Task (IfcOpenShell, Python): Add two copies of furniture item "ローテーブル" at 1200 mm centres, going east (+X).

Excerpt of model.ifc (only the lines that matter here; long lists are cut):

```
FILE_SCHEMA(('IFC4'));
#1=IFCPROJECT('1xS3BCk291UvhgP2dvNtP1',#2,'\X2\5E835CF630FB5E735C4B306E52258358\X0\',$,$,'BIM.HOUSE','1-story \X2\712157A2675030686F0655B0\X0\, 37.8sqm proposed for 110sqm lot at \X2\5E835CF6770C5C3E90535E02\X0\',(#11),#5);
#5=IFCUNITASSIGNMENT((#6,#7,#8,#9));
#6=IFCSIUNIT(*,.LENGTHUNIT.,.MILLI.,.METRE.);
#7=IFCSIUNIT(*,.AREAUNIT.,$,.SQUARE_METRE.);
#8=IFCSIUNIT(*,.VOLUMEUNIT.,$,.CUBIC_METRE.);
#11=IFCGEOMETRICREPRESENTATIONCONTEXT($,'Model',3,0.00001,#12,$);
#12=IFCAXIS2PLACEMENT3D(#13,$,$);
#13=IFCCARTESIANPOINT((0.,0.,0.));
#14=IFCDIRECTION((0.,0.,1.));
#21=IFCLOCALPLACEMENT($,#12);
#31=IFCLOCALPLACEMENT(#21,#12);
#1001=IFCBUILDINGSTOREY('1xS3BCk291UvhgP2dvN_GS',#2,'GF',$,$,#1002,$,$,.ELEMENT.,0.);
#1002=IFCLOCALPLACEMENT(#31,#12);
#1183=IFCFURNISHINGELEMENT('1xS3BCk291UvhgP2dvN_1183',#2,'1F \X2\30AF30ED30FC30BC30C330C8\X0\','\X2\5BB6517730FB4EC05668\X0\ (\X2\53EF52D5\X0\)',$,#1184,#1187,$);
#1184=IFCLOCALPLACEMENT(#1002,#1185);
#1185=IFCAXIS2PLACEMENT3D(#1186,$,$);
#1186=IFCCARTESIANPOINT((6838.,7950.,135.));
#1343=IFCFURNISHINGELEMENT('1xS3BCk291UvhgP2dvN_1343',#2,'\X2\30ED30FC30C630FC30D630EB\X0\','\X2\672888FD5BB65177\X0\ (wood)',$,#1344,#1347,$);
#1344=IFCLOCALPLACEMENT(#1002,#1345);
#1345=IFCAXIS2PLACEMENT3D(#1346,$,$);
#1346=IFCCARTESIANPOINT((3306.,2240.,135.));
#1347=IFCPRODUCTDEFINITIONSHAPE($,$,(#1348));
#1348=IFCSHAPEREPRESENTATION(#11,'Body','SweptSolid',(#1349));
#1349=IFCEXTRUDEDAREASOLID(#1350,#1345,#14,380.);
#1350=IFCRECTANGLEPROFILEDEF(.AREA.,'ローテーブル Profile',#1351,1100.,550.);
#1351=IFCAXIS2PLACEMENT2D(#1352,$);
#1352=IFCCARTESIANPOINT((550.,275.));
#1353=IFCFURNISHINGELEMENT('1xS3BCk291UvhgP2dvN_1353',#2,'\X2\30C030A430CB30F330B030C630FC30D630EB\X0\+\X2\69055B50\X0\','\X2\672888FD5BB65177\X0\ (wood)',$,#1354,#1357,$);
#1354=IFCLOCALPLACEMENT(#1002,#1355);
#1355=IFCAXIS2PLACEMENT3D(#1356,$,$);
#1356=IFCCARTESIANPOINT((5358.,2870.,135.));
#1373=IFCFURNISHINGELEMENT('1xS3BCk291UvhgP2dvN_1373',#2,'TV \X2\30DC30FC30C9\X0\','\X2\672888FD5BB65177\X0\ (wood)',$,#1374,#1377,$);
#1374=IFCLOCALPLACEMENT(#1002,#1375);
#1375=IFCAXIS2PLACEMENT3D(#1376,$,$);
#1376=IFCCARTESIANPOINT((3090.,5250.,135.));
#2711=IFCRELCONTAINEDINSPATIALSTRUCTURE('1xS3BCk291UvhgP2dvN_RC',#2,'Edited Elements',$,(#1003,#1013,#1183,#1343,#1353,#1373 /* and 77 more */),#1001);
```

```python
import numpy as np
import ifcopenshell
import ifcopenshell.api.geometry
import ifcopenshell.api.root
import ifcopenshell.util.element
import ifcopenshell.util.placement
import ifcopenshell.util.unit

model = ifcopenshell.open("model.ifc")
unit_scale = ifcopenshell.util.unit.calculate_unit_scale(model)


def reuse_history(source, copy):
    """copy_class also copies each property set's owner history, people and application; keep the originals."""
    for rel in copy.IsDefinedBy:
        if rel.is_a("IfcRelDefinesByProperties") and (history := rel.RelatingPropertyDefinition.OwnerHistory):
            rel.RelatingPropertyDefinition.OwnerHistory = source.OwnerHistory
            ifcopenshell.util.element.remove_deep2(model, history)


source = model.by_id(1343)
base = ifcopenshell.util.placement.get_local_placement(source.ObjectPlacement)
step = np.array([1.0, 0.0, 0.0]) * 1.2 / unit_scale

for i in range(1, 3):
    copy = ifcopenshell.api.root.copy_class(model, product=source)
    copy.Representation = ifcopenshell.util.element.copy_deep(
        model, source.Representation, exclude=["IfcGeometricRepresentationContext", "IfcRepresentationMap"]
    )
    reuse_history(source, copy)
    matrix = base.copy()
    matrix[:3, 3] += i * step
    print("added at", matrix[:3, 3].round(3) + 0.0)
    ifcopenshell.api.geometry.edit_object_placement(model, product=copy, matrix=matrix, is_si=False)

model.write("model_rev.ifc")
```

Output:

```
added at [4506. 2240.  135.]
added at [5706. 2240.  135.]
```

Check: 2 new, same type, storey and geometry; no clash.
